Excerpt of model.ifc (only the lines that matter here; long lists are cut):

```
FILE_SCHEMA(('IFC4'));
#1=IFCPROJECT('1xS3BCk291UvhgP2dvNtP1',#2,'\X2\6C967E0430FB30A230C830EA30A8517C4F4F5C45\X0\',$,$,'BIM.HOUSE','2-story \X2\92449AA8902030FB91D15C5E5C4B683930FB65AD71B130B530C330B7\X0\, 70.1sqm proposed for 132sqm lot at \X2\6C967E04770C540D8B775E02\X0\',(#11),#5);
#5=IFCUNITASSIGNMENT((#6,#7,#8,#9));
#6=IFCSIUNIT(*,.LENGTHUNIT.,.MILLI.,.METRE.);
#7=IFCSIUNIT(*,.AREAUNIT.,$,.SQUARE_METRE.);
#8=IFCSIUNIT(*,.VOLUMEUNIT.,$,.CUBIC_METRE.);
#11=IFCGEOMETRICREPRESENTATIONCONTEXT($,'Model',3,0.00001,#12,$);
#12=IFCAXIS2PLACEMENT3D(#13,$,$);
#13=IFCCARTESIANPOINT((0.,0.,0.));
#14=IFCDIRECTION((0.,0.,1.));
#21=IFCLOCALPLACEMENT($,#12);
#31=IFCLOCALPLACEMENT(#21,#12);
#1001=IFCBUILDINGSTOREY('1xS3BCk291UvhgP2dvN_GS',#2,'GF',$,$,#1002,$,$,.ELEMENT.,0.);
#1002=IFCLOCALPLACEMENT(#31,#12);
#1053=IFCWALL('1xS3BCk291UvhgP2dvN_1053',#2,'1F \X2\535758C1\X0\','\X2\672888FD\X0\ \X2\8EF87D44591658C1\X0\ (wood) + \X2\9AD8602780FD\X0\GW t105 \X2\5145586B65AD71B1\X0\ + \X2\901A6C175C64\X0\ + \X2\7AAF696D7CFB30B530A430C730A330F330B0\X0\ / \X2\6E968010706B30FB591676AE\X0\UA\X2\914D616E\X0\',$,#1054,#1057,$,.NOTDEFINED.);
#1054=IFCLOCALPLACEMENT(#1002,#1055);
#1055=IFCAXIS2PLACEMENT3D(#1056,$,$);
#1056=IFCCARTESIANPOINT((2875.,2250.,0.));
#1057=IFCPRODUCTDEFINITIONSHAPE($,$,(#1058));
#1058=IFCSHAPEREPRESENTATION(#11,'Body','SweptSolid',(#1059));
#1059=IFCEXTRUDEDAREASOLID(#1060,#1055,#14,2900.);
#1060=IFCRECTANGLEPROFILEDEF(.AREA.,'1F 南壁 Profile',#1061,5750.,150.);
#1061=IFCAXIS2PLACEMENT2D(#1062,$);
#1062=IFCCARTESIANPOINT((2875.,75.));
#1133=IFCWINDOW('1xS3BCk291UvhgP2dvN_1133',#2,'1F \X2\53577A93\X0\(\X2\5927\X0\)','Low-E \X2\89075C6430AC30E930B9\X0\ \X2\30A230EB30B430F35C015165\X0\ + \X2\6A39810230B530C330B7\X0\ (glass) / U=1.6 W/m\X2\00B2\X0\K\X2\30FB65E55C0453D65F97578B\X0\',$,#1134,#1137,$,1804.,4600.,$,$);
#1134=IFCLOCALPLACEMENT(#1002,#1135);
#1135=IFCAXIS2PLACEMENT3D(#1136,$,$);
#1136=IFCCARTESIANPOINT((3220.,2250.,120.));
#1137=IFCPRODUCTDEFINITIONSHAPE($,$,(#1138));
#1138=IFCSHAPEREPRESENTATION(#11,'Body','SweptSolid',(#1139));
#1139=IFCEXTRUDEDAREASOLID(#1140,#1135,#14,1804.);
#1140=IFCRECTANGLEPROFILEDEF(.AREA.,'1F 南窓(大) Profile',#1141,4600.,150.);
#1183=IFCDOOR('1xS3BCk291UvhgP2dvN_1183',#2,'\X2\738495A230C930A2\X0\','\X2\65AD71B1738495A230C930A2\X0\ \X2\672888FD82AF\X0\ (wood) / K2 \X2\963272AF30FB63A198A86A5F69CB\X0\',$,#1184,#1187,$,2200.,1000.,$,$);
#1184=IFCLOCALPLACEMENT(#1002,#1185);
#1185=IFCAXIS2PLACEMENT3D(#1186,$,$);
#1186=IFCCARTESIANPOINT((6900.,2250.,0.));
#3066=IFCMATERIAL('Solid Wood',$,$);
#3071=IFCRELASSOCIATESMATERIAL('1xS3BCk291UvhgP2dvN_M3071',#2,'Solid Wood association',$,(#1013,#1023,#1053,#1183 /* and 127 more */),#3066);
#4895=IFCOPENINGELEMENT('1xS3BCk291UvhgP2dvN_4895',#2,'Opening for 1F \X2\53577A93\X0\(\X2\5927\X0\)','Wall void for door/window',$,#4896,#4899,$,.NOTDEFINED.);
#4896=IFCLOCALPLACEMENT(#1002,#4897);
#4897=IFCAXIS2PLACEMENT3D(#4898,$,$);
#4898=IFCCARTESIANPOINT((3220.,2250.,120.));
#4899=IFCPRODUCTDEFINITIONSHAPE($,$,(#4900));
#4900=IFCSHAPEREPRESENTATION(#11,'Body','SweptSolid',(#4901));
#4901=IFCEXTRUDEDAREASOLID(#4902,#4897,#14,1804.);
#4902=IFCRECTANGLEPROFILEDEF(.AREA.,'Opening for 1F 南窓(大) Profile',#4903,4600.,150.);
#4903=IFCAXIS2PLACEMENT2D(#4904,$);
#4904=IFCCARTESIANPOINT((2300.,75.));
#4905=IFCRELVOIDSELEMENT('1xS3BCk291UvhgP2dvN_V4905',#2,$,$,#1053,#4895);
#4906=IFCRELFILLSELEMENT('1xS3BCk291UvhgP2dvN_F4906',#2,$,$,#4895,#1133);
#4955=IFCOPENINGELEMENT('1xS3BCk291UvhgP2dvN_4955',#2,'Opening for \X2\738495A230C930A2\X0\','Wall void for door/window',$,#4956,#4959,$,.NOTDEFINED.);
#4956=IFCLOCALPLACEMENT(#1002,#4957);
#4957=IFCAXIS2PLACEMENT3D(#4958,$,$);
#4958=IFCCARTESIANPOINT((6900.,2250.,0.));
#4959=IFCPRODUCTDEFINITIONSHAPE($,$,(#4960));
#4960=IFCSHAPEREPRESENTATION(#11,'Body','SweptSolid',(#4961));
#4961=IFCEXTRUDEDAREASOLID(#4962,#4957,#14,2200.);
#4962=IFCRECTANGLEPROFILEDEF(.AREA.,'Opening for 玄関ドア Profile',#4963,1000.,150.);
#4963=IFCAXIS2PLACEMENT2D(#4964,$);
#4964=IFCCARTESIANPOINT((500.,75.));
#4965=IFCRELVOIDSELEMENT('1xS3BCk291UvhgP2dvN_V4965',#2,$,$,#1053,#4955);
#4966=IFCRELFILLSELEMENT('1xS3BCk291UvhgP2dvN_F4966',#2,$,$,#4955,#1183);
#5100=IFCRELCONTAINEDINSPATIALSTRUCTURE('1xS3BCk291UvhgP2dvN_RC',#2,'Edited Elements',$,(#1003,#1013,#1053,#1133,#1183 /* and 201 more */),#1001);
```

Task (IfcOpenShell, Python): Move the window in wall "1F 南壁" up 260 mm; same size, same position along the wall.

```python
import numpy as np
import ifcopenshell
import ifcopenshell.api.geometry
import ifcopenshell.util.placement
import ifcopenshell.util.unit

model = ifcopenshell.open("model.ifc")
unit_scale = ifcopenshell.util.unit.calculate_unit_scale(model)

window = model.by_id(1133)
opening = window.FillsVoids[0].RelatingOpeningElement
dz = 260.0

shift = np.array([0.0, 0.0, dz])
# The window is not placed relative to its opening, so move both.
for product in (opening, window):
    matrix = ifcopenshell.util.placement.get_local_placement(product.ObjectPlacement)
    matrix[:3, 3] += shift
    ifcopenshell.api.geometry.edit_object_placement(model, product=product, matrix=matrix, is_si=False)

print(f"moved by {dz * unit_scale:+.3f} m")

model.write("model_updated.ifc")
```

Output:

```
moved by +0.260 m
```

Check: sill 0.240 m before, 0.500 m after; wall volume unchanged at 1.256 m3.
